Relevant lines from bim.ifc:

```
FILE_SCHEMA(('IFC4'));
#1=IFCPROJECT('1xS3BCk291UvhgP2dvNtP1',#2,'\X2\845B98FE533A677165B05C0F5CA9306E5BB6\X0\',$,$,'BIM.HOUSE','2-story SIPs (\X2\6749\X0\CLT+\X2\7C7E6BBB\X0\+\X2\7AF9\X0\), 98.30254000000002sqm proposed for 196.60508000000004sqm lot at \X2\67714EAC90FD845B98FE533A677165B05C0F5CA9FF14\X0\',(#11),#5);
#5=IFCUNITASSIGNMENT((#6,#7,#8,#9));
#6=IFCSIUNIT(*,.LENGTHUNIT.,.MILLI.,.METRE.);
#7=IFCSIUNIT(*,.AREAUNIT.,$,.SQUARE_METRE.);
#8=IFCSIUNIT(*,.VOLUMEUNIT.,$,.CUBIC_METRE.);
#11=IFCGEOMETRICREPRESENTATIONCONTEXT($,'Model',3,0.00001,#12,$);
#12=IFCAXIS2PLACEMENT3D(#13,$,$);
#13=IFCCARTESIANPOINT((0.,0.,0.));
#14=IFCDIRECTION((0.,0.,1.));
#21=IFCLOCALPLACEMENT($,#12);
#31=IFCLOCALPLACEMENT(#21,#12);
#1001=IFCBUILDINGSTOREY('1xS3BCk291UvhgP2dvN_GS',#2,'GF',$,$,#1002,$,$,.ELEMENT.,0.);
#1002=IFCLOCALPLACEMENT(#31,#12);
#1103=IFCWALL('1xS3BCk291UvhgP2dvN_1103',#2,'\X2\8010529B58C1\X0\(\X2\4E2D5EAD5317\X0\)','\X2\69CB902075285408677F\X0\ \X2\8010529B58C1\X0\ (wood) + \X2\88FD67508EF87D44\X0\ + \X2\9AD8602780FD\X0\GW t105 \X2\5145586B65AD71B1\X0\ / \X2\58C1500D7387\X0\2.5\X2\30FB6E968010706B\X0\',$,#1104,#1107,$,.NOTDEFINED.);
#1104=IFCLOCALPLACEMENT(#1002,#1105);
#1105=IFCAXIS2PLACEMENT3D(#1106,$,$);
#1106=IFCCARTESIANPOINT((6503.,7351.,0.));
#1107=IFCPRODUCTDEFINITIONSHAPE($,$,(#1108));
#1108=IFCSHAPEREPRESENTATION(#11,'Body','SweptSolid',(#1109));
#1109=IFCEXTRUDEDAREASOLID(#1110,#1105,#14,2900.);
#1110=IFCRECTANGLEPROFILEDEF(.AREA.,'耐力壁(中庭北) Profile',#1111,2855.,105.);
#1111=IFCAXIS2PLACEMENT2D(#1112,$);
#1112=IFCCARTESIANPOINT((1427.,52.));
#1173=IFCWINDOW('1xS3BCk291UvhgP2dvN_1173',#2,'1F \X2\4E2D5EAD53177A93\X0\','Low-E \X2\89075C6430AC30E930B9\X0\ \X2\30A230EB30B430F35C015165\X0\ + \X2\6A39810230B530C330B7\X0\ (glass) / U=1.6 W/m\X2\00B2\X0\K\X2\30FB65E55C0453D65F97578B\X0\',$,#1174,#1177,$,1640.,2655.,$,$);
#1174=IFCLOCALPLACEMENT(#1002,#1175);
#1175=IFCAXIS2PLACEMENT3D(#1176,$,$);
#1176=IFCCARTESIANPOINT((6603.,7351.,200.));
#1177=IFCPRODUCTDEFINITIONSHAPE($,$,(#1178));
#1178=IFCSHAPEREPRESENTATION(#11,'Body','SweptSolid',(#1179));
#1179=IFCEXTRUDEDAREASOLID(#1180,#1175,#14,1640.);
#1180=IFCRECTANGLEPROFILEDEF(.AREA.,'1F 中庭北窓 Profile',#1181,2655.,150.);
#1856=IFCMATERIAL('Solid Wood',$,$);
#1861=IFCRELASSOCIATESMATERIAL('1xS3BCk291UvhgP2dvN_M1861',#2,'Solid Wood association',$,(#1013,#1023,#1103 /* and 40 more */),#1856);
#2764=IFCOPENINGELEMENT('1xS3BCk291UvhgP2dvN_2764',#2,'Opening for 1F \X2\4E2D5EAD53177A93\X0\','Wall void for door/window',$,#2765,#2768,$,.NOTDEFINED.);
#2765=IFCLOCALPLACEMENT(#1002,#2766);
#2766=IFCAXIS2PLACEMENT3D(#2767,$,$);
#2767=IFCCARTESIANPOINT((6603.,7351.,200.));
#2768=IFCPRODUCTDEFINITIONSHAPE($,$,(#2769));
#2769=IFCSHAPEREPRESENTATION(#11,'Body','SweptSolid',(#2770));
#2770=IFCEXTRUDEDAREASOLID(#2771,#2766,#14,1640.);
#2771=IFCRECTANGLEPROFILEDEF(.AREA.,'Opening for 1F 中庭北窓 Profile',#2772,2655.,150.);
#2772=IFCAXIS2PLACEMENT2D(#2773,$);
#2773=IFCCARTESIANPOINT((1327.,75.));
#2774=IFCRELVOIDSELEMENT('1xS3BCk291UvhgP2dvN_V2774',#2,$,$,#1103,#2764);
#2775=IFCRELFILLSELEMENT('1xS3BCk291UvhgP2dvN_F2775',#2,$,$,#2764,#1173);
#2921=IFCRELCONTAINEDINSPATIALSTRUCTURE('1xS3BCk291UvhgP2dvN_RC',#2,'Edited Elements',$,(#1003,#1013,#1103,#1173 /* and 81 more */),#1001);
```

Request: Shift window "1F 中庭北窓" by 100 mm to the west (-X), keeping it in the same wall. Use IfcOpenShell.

```python
import ifcopenshell
import ifcopenshell.api.geometry
import ifcopenshell.util.placement

model = ifcopenshell.open("bim.ifc")

window = model.by_guid("1xS3BCk291UvhgP2dvN_1173")
opening = window.FillsVoids[0].RelatingOpeningElement
wall = opening.VoidsElements[0].RelatingBuildingElement

wall_matrix = ifcopenshell.util.placement.get_local_placement(wall.ObjectPlacement)
shift = wall_matrix[:3, 0] * -100.0
before = ifcopenshell.util.placement.get_local_placement(window.ObjectPlacement)[:3, 3].copy()

# The window is not placed relative to its opening, so move both.
for product in (opening, window):
    matrix = ifcopenshell.util.placement.get_local_placement(product.ObjectPlacement)
    matrix[:3, 3] += shift
    ifcopenshell.api.geometry.edit_object_placement(model, product=product, matrix=matrix, is_si=False)

after = ifcopenshell.util.placement.get_local_placement(window.ObjectPlacement)[:3, 3]
print("window moved by", (after - before).round(3) + 0.0)

model.write("bim_v2.ifc")
```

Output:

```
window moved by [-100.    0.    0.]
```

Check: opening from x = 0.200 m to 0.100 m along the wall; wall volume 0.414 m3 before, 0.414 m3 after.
